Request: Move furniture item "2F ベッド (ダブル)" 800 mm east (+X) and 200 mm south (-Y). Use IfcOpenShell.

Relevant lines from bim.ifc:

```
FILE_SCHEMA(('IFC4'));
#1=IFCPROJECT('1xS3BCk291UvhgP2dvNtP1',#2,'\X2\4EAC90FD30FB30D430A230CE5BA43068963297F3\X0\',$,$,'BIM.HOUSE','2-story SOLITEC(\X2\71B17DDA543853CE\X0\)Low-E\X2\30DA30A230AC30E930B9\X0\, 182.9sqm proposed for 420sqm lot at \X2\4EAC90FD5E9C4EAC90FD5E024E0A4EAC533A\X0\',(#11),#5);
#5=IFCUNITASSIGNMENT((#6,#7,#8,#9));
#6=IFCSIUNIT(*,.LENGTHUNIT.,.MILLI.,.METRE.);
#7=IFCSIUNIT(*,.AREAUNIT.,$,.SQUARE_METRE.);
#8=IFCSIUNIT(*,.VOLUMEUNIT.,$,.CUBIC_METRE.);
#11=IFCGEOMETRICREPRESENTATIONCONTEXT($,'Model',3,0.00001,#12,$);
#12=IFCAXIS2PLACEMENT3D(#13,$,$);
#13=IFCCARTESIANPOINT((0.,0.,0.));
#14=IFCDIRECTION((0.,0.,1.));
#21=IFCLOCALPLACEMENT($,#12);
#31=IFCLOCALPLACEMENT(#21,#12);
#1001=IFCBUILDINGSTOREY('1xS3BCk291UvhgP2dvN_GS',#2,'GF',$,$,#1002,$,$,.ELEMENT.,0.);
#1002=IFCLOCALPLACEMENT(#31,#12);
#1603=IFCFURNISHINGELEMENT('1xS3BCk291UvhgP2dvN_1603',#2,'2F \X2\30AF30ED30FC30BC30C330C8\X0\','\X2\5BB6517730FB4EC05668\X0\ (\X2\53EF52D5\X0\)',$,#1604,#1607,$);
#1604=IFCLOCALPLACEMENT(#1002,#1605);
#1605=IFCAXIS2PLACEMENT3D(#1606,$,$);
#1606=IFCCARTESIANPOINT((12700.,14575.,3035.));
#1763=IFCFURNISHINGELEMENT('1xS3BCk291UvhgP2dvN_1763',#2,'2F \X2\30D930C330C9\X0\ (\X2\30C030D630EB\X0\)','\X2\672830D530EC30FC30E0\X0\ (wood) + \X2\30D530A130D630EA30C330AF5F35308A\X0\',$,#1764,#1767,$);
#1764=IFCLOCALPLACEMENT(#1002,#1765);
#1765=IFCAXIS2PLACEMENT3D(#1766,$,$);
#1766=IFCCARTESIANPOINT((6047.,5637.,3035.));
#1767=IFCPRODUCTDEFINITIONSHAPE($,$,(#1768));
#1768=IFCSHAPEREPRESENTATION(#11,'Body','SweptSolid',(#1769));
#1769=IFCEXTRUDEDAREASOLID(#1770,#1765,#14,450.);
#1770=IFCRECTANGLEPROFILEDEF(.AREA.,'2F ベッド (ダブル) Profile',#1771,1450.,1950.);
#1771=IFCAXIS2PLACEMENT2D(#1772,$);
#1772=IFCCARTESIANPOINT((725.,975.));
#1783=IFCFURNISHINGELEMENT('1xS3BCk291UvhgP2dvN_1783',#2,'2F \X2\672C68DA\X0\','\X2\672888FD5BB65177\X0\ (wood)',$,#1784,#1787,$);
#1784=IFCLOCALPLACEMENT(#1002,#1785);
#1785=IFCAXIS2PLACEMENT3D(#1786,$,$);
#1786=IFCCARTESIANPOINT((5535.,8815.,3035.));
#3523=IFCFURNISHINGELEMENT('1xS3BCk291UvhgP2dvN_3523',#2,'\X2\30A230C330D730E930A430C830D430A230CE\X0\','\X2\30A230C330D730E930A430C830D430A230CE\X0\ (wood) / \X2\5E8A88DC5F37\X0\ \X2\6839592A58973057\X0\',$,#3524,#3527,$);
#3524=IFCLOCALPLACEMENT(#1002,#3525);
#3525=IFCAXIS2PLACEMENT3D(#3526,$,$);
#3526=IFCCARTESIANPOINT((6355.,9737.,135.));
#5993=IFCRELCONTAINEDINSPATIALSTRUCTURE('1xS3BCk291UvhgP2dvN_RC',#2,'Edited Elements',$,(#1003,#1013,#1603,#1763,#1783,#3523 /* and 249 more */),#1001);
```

```python
import ifcopenshell
import ifcopenshell.api.geometry
import ifcopenshell.util.placement
import ifcopenshell.util.unit

model = ifcopenshell.open("bim.ifc")
unit_scale = ifcopenshell.util.unit.calculate_unit_scale(model)

item = model.by_guid("1xS3BCk291UvhgP2dvN_1763")
matrix = ifcopenshell.util.placement.get_local_placement(item.ObjectPlacement)
matrix[0, 3] += 0.8 / unit_scale
matrix[1, 3] -= 0.2 / unit_scale
ifcopenshell.api.geometry.edit_object_placement(model, product=item, matrix=matrix, is_si=False)

print(ifcopenshell.util.placement.get_local_placement(item.ObjectPlacement).round(3) + 0.0)

model.write("bim_updated.ifc")
```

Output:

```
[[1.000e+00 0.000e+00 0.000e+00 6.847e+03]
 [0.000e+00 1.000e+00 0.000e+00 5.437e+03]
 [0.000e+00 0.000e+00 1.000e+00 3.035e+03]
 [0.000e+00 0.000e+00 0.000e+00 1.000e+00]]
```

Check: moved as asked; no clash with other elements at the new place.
